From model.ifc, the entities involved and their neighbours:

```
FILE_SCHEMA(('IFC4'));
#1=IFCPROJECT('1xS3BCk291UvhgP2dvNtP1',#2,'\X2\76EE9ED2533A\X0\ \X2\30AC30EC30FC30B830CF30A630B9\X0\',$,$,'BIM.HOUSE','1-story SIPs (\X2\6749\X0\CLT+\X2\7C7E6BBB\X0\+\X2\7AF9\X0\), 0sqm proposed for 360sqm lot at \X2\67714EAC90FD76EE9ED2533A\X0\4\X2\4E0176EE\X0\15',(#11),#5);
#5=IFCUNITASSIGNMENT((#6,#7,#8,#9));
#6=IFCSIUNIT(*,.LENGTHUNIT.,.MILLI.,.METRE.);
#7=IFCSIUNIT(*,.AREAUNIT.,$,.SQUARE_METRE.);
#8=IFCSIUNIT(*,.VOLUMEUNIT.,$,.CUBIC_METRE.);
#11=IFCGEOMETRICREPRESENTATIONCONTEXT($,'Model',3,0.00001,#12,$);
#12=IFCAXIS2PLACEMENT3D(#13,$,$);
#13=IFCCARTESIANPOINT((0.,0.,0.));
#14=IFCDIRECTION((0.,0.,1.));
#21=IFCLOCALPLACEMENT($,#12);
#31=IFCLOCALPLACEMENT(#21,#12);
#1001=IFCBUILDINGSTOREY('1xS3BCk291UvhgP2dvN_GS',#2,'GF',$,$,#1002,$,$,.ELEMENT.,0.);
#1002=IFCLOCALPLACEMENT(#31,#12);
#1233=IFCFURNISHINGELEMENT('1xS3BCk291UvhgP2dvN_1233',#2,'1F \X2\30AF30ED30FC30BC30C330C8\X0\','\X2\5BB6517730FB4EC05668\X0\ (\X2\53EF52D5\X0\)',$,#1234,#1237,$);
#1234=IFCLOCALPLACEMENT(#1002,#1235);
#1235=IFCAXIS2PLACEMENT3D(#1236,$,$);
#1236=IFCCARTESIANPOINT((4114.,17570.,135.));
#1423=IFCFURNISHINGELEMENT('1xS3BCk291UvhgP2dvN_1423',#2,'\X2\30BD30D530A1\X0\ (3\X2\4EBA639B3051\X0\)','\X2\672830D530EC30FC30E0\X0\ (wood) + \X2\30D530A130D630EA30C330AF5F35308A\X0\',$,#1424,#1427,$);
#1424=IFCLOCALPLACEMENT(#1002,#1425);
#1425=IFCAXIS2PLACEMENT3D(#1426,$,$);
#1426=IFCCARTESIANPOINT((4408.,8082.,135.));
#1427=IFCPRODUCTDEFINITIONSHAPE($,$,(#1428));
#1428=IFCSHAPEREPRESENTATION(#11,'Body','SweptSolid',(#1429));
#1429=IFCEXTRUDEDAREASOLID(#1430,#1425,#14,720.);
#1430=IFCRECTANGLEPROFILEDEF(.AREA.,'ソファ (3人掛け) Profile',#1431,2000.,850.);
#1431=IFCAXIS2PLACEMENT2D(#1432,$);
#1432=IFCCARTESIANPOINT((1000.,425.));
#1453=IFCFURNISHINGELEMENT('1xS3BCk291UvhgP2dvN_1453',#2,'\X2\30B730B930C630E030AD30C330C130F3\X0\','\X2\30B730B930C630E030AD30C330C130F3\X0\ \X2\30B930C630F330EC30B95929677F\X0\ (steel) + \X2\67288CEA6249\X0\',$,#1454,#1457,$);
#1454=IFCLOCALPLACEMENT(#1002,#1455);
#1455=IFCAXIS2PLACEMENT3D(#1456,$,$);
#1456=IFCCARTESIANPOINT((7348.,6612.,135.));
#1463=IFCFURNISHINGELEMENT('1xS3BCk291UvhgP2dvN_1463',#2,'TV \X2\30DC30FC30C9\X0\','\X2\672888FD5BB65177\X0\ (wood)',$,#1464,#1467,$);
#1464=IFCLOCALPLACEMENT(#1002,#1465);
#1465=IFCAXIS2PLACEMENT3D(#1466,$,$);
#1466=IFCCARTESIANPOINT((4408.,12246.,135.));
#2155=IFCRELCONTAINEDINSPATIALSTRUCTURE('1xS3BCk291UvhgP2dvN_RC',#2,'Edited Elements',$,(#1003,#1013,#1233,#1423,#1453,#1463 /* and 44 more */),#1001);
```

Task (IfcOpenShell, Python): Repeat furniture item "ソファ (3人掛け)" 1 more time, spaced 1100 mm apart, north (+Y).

```python
import numpy as np
import ifcopenshell
import ifcopenshell.api.geometry
import ifcopenshell.api.root
import ifcopenshell.util.element
import ifcopenshell.util.placement

model = ifcopenshell.open("model.ifc")


def reuse_history(source, copy):
    """copy_class also copies each property set's owner history, people and application; keep the originals."""
    for rel in copy.IsDefinedBy:
        if rel.is_a("IfcRelDefinesByProperties") and (history := rel.RelatingPropertyDefinition.OwnerHistory):
            rel.RelatingPropertyDefinition.OwnerHistory = source.OwnerHistory
            ifcopenshell.util.element.remove_deep2(model, history)


source = model.by_guid("1xS3BCk291UvhgP2dvN_1423")
base = ifcopenshell.util.placement.get_local_placement(source.ObjectPlacement)
step = np.array([0.0, 1.0, 0.0]) * 1100.0

for i in range(1, 2):
    copy = ifcopenshell.api.root.copy_class(model, product=source)
    copy.Representation = ifcopenshell.util.element.copy_deep(
        model, source.Representation, exclude=["IfcGeometricRepresentationContext", "IfcRepresentationMap"]
    )
    reuse_history(source, copy)
    matrix = base.copy()
    matrix[:3, 3] += i * step
    print("added at", matrix[:3, 3].round(3) + 0.0)
    ifcopenshell.api.geometry.edit_object_placement(model, product=copy, matrix=matrix, is_si=False)

model.write("model_v2.ifc")
```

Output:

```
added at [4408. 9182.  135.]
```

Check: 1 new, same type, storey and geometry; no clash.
